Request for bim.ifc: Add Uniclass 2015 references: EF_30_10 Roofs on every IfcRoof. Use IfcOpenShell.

First a look at what the model holds.

```python
import ifcopenshell

model = ifcopenshell.open("bim.ifc")
print(model.schema)
print("classifications:", [c.Name for c in model.by_type("IfcClassification")])
for ifc_class in ("IfcDoor", "IfcRoof", "IfcStair", "IfcWall", "IfcWindow"):
    print(ifc_class, len(model.by_type(ifc_class)))
```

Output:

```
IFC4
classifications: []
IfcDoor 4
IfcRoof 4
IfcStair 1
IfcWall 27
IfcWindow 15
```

```python
import ifcopenshell
import ifcopenshell.api.classification

model = ifcopenshell.open("bim.ifc")

system = ifcopenshell.api.classification.add_classification(model, classification="Uniclass 2015")

codes = {
    "IfcRoof": ("EF_30_10", "Roofs"),
}
for ifc_class, (code, name) in codes.items():
    products = model.by_type(ifc_class)
    ifcopenshell.api.classification.add_reference(
        model, products=products, classification=system, identification=code, name=name
    )
    print(code, len(products))

model.write("bim_edited.ifc")
```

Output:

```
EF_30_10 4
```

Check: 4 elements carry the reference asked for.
